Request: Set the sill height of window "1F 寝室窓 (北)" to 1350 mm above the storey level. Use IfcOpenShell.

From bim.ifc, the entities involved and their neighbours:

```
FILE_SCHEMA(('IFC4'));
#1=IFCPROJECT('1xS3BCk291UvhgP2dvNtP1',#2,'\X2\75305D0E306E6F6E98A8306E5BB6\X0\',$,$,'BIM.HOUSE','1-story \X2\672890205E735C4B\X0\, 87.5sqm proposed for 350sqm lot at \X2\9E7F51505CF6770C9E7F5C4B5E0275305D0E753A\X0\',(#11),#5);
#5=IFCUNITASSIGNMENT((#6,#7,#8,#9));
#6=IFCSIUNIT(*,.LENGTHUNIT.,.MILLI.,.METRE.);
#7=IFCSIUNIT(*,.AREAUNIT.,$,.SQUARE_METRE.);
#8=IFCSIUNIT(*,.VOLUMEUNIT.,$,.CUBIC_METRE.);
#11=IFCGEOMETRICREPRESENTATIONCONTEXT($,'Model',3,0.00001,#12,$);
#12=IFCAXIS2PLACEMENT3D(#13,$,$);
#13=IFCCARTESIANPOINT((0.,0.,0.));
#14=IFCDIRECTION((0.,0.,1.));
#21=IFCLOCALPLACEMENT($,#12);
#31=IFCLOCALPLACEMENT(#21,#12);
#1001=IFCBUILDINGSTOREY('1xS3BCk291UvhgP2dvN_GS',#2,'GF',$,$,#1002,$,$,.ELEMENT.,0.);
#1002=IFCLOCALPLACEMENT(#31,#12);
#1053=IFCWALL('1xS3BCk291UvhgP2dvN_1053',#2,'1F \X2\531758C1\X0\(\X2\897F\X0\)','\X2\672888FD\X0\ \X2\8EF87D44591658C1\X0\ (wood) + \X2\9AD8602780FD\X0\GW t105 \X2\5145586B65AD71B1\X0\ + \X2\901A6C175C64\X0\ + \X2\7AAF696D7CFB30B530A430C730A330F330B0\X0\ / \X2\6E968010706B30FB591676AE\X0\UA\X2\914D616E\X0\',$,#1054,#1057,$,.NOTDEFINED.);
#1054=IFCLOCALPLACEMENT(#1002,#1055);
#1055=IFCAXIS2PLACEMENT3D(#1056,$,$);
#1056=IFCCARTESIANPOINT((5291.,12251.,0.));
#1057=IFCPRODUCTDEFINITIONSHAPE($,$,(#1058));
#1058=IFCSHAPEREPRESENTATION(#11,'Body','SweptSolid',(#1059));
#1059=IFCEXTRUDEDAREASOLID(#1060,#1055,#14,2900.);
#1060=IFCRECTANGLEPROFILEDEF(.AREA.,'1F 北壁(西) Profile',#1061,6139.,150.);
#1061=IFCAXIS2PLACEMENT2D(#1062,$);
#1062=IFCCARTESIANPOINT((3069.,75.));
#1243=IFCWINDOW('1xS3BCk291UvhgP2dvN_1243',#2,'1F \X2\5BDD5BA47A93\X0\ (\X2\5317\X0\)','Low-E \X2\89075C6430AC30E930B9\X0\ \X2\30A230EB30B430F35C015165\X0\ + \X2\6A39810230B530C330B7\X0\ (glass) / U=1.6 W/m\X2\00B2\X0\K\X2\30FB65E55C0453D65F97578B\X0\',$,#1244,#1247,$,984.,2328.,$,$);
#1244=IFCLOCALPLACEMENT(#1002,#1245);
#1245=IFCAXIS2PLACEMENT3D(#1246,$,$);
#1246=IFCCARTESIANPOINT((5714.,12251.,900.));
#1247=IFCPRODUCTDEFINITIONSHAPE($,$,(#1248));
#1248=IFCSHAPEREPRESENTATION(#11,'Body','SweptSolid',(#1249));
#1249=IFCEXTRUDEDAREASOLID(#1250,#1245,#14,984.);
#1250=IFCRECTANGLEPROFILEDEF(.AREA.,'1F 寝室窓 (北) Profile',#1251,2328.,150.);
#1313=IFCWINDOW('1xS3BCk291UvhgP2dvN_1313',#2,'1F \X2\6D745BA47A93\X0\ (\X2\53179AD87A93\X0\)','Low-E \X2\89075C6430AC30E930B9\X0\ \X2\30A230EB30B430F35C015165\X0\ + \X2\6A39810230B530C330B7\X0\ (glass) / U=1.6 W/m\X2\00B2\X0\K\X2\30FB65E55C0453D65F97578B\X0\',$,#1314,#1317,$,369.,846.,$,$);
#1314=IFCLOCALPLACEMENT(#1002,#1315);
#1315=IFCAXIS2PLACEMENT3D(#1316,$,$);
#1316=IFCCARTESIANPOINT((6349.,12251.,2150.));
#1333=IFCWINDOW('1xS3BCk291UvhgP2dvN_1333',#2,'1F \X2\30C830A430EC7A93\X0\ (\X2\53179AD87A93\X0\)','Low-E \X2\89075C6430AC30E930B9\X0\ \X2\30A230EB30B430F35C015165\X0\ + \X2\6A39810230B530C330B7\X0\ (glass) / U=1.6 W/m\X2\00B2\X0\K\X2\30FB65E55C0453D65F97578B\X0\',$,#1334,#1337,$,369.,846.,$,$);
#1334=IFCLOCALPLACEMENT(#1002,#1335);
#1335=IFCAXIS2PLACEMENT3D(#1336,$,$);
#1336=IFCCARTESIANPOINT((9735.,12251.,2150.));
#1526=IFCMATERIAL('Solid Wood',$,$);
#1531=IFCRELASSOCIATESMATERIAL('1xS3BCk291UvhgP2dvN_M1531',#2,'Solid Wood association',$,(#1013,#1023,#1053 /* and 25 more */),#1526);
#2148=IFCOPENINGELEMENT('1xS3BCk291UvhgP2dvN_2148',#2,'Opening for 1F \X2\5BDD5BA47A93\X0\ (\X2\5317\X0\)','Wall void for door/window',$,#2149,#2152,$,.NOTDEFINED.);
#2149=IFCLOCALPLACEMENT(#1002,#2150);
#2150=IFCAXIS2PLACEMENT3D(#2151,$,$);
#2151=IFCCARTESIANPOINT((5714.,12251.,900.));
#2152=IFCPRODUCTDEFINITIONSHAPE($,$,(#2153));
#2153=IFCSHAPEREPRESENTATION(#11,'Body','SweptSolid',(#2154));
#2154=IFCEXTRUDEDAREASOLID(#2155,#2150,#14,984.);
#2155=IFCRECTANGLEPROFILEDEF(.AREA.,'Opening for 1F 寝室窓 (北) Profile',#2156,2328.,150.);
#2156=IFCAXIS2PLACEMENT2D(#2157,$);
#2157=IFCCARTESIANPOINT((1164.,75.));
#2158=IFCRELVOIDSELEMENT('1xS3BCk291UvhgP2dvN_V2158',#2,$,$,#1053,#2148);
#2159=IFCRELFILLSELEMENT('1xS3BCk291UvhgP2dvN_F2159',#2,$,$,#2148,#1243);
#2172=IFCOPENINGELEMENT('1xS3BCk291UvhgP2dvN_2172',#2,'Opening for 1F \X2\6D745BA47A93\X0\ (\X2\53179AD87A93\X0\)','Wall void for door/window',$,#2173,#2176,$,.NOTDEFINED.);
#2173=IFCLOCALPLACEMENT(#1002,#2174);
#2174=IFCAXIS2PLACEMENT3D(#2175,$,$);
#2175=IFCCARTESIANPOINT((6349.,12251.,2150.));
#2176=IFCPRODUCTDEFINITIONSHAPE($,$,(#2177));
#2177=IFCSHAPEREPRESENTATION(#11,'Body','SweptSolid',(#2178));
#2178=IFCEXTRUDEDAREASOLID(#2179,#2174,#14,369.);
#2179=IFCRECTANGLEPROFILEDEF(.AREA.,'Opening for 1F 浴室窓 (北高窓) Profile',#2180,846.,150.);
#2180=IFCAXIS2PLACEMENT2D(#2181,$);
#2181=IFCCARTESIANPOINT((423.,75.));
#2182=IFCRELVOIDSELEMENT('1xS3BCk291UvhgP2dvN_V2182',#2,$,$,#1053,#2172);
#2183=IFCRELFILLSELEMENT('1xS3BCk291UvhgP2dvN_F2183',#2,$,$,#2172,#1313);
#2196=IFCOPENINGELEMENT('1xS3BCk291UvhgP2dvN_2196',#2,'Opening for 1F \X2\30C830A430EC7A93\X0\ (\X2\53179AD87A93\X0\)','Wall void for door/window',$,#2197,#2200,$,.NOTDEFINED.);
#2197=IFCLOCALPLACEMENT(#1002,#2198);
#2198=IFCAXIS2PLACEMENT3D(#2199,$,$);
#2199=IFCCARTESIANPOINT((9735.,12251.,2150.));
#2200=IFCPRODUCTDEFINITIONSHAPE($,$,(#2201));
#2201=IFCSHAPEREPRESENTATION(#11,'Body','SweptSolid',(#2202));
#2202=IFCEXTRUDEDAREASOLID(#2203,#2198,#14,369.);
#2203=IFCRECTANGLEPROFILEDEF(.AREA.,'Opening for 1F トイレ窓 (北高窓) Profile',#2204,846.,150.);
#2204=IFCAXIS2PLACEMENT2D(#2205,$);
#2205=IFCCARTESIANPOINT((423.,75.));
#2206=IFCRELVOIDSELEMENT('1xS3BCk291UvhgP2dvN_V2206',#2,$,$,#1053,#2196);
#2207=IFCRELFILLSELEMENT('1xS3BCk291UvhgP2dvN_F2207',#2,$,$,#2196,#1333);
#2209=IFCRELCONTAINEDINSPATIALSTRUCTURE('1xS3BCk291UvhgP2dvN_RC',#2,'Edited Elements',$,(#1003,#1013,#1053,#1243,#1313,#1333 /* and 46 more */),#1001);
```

```python
import numpy as np
import ifcopenshell
import ifcopenshell.api.geometry
import ifcopenshell.geom
import ifcopenshell.util.element
import ifcopenshell.util.placement
import ifcopenshell.util.shape
import ifcopenshell.util.unit

model = ifcopenshell.open("bim.ifc")
unit_scale = ifcopenshell.util.unit.calculate_unit_scale(model)

window = model.by_guid("1xS3BCk291UvhgP2dvN_1243")
opening = window.FillsVoids[0].RelatingOpeningElement
storey = ifcopenshell.util.element.get_container(window, ifc_class="IfcBuildingStorey")
level = ifcopenshell.util.placement.get_local_placement(storey.ObjectPlacement)[2, 3]

# The opening's origin need not be at the sill, so measure its lowest point.
shape = ifcopenshell.geom.create_shape(ifcopenshell.geom.settings(), opening)
bottom = ifcopenshell.util.shape.get_shape_bottom_elevation(shape, shape.geometry) / unit_scale
dz = level + 1.35 / unit_scale - bottom

shift = np.array([0.0, 0.0, dz])
# The window is not placed relative to its opening, so move both.
for product in (opening, window):
    matrix = ifcopenshell.util.placement.get_local_placement(product.ObjectPlacement)
    matrix[:3, 3] += shift
    ifcopenshell.api.geometry.edit_object_placement(model, product=product, matrix=matrix, is_si=False)

print(f"moved by {dz * unit_scale:+.3f} m")

model.write("bim_v2.ifc")
```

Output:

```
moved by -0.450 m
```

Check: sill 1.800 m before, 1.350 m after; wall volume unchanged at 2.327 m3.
